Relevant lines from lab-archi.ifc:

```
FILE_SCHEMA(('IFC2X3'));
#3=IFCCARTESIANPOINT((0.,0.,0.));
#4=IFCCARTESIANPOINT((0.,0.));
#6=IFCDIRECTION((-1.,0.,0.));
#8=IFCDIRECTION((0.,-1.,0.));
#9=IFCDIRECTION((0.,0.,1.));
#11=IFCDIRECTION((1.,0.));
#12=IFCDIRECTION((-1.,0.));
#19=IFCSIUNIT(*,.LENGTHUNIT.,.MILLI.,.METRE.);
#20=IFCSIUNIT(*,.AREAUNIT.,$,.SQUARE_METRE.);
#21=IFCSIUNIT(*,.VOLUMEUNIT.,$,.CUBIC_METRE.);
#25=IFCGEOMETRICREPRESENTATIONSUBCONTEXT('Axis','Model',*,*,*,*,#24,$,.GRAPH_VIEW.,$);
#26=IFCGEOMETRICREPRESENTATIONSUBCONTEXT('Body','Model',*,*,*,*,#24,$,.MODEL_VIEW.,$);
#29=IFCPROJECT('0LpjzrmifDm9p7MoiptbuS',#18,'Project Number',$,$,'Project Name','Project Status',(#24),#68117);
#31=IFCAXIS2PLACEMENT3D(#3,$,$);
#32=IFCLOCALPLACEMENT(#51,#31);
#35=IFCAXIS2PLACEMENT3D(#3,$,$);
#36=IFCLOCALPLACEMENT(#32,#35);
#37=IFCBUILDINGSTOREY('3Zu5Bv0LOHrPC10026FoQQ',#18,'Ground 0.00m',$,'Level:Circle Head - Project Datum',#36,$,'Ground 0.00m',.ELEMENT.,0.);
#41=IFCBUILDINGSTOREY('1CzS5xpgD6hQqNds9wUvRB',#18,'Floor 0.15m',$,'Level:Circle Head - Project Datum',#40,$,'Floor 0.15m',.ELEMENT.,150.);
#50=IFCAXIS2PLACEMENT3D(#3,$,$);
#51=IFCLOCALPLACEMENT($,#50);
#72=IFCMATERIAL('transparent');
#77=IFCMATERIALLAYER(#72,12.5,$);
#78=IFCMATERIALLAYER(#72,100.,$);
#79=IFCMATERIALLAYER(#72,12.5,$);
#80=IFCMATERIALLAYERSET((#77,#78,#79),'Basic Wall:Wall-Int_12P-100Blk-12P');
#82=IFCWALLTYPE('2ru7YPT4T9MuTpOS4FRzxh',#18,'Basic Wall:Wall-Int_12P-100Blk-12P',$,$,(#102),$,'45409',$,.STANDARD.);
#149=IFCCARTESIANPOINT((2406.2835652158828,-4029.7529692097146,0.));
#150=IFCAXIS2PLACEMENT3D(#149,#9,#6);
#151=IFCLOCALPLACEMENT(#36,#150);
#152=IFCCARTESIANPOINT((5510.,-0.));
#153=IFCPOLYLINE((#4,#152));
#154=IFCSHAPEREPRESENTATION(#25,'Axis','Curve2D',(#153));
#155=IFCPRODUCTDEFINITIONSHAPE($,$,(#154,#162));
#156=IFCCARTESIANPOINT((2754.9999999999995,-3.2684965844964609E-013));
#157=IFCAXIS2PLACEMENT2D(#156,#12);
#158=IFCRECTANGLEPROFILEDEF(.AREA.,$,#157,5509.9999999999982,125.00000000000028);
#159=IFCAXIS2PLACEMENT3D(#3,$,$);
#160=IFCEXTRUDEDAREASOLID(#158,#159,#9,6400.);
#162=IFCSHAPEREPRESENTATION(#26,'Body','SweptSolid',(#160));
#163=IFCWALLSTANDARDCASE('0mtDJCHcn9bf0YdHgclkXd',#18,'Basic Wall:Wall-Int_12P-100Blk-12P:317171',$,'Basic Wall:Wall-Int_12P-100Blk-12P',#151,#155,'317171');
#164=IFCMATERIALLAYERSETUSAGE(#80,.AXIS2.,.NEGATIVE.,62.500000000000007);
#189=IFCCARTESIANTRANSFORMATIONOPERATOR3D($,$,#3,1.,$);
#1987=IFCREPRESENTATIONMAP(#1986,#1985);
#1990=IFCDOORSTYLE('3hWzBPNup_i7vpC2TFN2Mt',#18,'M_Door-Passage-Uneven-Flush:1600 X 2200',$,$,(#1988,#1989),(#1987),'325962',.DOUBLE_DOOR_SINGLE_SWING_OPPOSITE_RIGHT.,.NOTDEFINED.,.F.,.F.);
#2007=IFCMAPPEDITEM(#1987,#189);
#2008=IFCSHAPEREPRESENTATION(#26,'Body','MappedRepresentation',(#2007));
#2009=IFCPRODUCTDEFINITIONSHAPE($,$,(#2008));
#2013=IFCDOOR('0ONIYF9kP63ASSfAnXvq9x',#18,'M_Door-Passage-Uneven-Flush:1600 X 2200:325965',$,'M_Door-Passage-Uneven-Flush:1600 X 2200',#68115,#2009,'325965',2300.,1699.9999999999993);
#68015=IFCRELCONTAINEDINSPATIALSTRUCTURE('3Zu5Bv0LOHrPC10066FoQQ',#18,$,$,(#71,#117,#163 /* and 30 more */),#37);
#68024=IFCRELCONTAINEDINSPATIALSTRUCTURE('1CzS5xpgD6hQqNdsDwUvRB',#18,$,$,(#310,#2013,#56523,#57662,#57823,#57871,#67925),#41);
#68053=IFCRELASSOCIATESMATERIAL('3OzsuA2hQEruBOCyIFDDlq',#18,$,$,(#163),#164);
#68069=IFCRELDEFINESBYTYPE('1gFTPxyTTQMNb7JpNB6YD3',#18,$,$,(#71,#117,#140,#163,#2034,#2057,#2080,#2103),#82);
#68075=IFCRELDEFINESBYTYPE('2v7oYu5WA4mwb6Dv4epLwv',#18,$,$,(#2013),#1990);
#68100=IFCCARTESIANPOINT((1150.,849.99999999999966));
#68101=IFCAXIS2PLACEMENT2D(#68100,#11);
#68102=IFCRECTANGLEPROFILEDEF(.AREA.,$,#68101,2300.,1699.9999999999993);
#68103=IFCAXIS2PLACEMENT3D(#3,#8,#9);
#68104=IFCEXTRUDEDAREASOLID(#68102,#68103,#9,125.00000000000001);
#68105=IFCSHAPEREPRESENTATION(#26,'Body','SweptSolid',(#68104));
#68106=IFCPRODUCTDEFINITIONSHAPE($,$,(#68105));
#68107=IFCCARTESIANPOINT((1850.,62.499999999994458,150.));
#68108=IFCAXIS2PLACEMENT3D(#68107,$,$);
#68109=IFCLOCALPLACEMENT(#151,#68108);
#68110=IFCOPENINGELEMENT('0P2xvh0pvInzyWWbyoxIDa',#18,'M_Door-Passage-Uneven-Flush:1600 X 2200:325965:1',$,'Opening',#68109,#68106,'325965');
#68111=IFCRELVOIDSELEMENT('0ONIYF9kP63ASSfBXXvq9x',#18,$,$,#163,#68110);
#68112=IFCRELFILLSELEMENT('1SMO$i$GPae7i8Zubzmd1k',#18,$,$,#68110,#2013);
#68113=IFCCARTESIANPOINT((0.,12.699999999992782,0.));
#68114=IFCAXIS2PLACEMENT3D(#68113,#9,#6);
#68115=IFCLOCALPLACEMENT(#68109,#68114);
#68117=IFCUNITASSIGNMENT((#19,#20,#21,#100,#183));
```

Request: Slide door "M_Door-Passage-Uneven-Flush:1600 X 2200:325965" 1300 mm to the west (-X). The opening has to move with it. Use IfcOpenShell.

```python
import ifcopenshell
import ifcopenshell.api.geometry
import ifcopenshell.util.placement
import ifcopenshell.util.unit

model = ifcopenshell.open("lab-archi.ifc")
unit_scale = ifcopenshell.util.unit.calculate_unit_scale(model)

door = model.by_id(2013)
opening = door.FillsVoids[0].RelatingOpeningElement
wall = opening.VoidsElements[0].RelatingBuildingElement

wall_matrix = ifcopenshell.util.placement.get_local_placement(wall.ObjectPlacement)
shift = wall_matrix[:3, 0] * 1.3 / unit_scale
before = ifcopenshell.util.placement.get_local_placement(door.ObjectPlacement)[:3, 3].copy()

# The door is placed relative to its opening, so it follows when the opening moves.
matrix = ifcopenshell.util.placement.get_local_placement(opening.ObjectPlacement)
matrix[:3, 3] += shift
ifcopenshell.api.geometry.edit_object_placement(
    model, product=opening, matrix=matrix, is_si=False, should_transform_children=True
)

after = ifcopenshell.util.placement.get_local_placement(door.ObjectPlacement)[:3, 3]
print("door moved by", (after - before).round(3) + 0.0)

model.write("lab-archi-out.ifc")
```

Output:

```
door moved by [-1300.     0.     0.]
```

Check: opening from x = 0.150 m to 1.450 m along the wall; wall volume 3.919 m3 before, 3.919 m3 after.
